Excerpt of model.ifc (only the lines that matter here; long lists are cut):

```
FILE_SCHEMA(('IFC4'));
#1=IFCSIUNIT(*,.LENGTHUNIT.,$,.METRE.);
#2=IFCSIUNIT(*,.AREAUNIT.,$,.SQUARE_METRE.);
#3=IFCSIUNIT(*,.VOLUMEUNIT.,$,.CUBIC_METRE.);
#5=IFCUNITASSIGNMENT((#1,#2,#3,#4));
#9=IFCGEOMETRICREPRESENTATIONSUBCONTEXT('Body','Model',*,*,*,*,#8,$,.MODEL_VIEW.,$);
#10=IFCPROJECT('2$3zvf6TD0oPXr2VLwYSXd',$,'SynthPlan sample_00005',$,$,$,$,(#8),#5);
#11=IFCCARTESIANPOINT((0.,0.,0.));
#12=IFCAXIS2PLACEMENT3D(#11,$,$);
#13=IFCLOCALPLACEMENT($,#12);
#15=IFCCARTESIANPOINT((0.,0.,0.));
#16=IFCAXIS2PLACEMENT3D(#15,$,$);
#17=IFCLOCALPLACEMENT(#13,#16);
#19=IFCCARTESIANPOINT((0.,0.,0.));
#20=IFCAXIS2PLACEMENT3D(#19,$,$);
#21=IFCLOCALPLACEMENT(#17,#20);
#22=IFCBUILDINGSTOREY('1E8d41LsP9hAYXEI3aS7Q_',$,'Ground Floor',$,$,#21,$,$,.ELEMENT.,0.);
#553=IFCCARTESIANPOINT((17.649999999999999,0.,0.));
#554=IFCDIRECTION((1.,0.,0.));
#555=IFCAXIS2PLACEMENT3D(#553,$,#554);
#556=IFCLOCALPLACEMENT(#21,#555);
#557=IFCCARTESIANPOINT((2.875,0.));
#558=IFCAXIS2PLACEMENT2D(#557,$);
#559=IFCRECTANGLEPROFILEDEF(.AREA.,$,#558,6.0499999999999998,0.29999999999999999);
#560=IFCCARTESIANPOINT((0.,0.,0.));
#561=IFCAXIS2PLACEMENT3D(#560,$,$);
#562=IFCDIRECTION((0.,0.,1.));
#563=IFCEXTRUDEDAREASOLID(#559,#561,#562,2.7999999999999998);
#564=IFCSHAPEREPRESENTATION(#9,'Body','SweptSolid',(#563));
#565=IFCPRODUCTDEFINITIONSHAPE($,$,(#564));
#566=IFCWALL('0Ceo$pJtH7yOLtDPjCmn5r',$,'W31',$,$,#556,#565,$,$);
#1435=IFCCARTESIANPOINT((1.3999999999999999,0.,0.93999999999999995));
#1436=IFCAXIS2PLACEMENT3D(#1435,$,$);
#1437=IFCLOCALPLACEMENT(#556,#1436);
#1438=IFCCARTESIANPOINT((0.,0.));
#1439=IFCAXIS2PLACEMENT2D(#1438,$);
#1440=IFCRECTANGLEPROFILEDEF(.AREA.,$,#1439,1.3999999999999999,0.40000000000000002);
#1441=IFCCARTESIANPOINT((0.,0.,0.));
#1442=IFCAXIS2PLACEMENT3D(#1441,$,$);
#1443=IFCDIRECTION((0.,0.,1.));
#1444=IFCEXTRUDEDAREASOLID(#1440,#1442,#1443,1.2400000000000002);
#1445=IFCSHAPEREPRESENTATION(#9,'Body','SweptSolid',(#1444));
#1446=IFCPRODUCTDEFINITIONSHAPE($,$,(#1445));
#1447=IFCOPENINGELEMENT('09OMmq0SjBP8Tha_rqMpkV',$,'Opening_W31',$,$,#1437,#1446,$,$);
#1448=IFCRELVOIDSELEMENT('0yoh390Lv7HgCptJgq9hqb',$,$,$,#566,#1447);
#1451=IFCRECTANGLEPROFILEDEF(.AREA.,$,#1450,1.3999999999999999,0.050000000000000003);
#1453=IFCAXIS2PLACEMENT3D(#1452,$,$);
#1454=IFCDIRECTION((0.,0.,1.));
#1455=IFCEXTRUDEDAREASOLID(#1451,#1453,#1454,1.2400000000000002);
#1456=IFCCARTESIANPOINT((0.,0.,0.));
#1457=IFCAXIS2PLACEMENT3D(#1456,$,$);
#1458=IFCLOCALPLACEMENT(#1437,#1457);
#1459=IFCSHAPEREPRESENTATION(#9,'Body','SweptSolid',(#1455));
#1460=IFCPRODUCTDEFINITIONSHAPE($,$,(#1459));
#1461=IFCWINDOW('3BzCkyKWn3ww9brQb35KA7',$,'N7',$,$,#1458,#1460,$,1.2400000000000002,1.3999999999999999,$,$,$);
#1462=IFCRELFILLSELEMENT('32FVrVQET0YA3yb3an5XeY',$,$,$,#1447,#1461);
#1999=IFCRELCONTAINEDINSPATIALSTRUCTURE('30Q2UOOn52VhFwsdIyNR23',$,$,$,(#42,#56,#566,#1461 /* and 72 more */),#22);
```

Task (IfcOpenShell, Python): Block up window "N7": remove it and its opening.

```python
import ifcopenshell
import ifcopenshell.api.feature
import ifcopenshell.api.root
import ifcopenshell.geom
import ifcopenshell.util.shape

model = ifcopenshell.open("model.ifc")
settings = ifcopenshell.geom.settings()


def volume(element):
    """Net volume in cubic metres, openings subtracted."""
    shape = ifcopenshell.geom.create_shape(settings, element)
    return ifcopenshell.util.shape.get_volume(shape.geometry)


window = model.by_id(1461)
opening = window.FillsVoids[0].RelatingOpeningElement
wall = opening.VoidsElements[0].RelatingBuildingElement
before = volume(wall)

ifcopenshell.api.root.remove_product(model, product=window)
ifcopenshell.api.feature.remove_feature(model, feature=opening)

after = volume(wall)

print(f"wall volume {before:.3f} -> {after:.3f} m3")

model.write("model_rev.ifc")
```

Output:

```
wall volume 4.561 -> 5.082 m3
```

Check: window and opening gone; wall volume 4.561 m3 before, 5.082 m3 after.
